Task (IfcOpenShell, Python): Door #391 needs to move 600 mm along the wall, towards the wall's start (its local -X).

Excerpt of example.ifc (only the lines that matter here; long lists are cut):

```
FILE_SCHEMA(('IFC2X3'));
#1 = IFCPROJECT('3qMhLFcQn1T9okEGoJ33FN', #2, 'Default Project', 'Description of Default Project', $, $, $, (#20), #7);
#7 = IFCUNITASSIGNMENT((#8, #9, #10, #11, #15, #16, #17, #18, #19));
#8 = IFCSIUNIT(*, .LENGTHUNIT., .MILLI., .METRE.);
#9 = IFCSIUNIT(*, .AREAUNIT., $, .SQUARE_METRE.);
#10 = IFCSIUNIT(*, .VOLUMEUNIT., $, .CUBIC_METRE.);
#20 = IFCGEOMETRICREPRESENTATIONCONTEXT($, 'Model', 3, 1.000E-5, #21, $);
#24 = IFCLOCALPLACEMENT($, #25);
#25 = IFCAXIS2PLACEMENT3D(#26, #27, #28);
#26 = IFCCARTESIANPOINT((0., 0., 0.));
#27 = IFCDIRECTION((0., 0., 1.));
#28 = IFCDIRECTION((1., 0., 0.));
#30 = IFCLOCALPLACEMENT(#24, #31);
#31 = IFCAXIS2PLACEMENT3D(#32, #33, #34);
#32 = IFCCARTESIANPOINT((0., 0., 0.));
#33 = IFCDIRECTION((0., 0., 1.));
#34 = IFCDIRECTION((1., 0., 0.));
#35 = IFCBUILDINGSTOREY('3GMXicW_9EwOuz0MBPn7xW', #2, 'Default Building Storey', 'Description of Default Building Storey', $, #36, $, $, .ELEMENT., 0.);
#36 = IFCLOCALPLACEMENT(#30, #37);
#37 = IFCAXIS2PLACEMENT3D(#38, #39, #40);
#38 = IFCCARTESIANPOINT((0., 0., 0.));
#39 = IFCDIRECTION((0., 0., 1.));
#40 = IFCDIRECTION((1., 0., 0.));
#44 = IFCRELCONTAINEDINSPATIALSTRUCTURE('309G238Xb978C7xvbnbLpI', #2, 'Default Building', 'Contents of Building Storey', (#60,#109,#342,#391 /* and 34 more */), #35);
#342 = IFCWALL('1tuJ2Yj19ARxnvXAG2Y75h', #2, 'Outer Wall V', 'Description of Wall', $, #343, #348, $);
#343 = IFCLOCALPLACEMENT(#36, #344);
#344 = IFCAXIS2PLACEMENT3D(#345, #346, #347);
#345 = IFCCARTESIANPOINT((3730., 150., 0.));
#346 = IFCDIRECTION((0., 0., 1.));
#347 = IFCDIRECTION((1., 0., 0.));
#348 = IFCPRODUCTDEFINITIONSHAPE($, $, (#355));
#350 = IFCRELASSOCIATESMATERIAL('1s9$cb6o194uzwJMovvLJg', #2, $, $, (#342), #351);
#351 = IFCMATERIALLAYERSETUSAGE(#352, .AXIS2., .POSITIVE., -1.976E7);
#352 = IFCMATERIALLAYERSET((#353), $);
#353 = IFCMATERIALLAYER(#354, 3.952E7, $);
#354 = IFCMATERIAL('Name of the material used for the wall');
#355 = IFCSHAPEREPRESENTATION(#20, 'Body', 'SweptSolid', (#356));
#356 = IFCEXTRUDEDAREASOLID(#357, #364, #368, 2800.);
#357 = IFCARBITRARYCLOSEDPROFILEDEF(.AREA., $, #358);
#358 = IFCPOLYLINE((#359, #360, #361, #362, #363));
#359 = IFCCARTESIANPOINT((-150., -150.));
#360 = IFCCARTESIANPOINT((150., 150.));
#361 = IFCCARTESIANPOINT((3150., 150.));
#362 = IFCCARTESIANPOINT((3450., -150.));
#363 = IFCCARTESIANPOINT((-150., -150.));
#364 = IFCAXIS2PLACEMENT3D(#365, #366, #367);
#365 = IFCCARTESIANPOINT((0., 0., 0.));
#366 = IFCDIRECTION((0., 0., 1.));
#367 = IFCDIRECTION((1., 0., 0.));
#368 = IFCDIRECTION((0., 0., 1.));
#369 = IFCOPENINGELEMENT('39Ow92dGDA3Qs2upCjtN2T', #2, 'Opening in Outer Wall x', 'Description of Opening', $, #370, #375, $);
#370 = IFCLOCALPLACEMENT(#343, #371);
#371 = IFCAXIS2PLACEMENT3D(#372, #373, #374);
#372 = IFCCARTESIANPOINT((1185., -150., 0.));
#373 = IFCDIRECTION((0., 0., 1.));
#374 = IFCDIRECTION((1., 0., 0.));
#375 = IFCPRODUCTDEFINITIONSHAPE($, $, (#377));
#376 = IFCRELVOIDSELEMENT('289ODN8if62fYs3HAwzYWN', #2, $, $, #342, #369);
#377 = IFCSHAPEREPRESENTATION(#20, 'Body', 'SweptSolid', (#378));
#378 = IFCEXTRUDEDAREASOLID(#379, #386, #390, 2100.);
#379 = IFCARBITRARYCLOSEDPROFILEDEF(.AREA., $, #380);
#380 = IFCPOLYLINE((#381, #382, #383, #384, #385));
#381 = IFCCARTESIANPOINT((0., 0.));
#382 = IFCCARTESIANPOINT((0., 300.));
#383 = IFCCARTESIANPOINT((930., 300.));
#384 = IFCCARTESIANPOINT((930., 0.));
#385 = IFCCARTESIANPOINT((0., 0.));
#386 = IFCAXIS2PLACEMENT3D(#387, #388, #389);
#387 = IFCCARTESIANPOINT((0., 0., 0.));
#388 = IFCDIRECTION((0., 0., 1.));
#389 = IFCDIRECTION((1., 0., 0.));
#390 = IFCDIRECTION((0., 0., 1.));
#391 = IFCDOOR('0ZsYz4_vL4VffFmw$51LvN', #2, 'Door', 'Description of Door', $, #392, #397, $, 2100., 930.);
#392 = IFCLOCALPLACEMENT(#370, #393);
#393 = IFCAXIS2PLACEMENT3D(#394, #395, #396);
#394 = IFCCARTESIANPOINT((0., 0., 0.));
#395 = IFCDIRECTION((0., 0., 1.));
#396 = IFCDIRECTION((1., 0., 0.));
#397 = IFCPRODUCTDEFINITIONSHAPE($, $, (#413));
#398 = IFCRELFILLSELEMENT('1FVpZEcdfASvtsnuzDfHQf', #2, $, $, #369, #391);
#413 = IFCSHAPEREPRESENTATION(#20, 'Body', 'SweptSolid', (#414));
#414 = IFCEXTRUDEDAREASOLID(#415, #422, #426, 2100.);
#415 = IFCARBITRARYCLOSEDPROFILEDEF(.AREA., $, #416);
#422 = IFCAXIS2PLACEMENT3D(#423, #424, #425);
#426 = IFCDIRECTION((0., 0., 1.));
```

```python
import ifcopenshell
import ifcopenshell.api.geometry
import ifcopenshell.util.placement
import ifcopenshell.util.unit

model = ifcopenshell.open("example.ifc")
unit_scale = ifcopenshell.util.unit.calculate_unit_scale(model)

door = model.by_guid("0ZsYz4_vL4VffFmw$51LvN")
opening = door.FillsVoids[0].RelatingOpeningElement
wall = opening.VoidsElements[0].RelatingBuildingElement

wall_matrix = ifcopenshell.util.placement.get_local_placement(wall.ObjectPlacement)
shift = wall_matrix[:3, 0] * -0.6 / unit_scale
before = ifcopenshell.util.placement.get_local_placement(door.ObjectPlacement)[:3, 3].copy()

# The door is placed relative to its opening, so it follows when the opening moves.
matrix = ifcopenshell.util.placement.get_local_placement(opening.ObjectPlacement)
matrix[:3, 3] += shift
ifcopenshell.api.geometry.edit_object_placement(
    model, product=opening, matrix=matrix, is_si=False, should_transform_children=True
)

after = ifcopenshell.util.placement.get_local_placement(door.ObjectPlacement)[:3, 3]
print("door moved by", (after - before).round(3) + 0.0)

model.write("example-out.ifc")
```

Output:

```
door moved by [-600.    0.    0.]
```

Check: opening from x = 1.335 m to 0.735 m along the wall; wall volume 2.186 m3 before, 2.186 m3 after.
